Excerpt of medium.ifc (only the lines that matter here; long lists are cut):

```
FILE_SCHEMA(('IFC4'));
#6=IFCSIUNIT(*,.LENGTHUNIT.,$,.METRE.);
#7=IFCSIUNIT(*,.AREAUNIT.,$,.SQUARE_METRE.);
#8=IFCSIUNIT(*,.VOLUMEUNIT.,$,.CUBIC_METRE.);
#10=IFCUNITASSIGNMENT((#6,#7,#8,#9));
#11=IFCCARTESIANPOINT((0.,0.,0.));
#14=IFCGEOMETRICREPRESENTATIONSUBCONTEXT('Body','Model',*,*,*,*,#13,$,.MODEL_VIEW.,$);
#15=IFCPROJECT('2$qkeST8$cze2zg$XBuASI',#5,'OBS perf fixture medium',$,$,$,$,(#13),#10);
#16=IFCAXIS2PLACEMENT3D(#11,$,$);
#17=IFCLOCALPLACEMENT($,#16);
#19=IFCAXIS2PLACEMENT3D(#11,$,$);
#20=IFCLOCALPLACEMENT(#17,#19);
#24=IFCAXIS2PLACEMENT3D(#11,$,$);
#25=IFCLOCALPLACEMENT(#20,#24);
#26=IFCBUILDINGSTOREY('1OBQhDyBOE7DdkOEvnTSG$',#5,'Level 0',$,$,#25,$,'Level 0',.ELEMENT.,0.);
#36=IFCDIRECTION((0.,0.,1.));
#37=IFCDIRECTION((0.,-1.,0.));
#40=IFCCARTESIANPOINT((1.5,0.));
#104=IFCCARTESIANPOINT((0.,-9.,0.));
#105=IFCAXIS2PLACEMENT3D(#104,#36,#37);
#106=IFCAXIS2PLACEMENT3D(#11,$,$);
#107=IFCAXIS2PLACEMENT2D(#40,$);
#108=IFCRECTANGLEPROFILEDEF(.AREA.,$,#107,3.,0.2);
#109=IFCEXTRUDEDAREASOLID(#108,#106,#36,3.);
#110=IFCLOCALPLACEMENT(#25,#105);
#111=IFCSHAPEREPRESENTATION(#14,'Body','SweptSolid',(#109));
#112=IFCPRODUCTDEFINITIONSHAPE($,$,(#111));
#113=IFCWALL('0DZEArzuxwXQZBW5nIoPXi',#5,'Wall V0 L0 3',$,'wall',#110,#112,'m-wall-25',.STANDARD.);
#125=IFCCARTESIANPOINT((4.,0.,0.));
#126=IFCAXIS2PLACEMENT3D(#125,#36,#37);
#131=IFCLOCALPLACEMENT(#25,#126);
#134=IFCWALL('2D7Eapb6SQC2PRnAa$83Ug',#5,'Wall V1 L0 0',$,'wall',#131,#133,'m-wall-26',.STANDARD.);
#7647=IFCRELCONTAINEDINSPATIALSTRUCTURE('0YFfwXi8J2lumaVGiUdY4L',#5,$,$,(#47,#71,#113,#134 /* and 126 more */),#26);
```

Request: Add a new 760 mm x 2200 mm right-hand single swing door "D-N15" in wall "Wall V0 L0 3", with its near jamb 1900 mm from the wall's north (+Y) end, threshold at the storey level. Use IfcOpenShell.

```python
import numpy as np
import ifcopenshell
import ifcopenshell.api.feature
import ifcopenshell.api.geometry
import ifcopenshell.api.root
import ifcopenshell.api.spatial
import ifcopenshell.geom
import ifcopenshell.util.element
import ifcopenshell.util.placement
import ifcopenshell.util.representation
import ifcopenshell.util.shape
import ifcopenshell.util.unit

model = ifcopenshell.open("medium.ifc")
unit_scale = ifcopenshell.util.unit.calculate_unit_scale(model)
settings = ifcopenshell.geom.settings()


def volume(element):
    """Net volume in cubic metres, openings subtracted."""
    shape = ifcopenshell.geom.create_shape(settings, element)
    return ifcopenshell.util.shape.get_volume(shape.geometry)


wall = model.by_guid("0DZEArzuxwXQZBW5nIoPXi")
storey = ifcopenshell.util.element.get_container(wall, ifc_class="IfcBuildingStorey")
context = ifcopenshell.util.representation.get_context(model, "Model", "Body", "MODEL_VIEW")
before = volume(wall)

width, height, from_end, sill = 0.76, 2.2, 1.9, 0.0  # metres

# The wall runs along its own X axis, and the end named is its -X end.
wall_shape = ifcopenshell.geom.create_shape(settings, wall)
x, y, z = ifcopenshell.util.shape.get_vertices(wall_shape.geometry).T
start = x.min() + from_end
face, thickness = float(y.min()), float(y.max() - y.min())
wall_matrix = ifcopenshell.util.placement.get_local_placement(wall.ObjectPlacement)
level = ifcopenshell.util.placement.get_local_placement(storey.ObjectPlacement)[2, 3]


def in_wall(x, y):
    """Placement at x, y metres in the wall's axes, at sill height."""
    matrix = wall_matrix.copy()
    matrix[:, 3] = wall_matrix @ np.array([x / unit_scale, y / unit_scale, 0.0, 1.0])
    matrix[2, 3] = level + sill / unit_scale
    return matrix


# Opening: a box that overshoots both wall faces by 50 mm.
opening = ifcopenshell.api.root.create_entity(model, ifc_class="IfcOpeningElement", predefined_type="OPENING")
box = ifcopenshell.api.geometry.add_wall_representation(
    model, context=context, length=width, height=height, thickness=thickness + 0.1
)
ifcopenshell.api.geometry.assign_representation(model, product=opening, representation=box)
ifcopenshell.api.geometry.edit_object_placement(model, product=opening, matrix=in_wall(start, face - 0.05), is_si=False)
ifcopenshell.api.feature.add_feature(model, feature=opening, element=wall)

door = ifcopenshell.api.root.create_entity(model, ifc_class="IfcDoor", name="D-N15", predefined_type="DOOR")
door.OverallWidth, door.OverallHeight = width / unit_scale, height / unit_scale
door.OperationType = "SINGLE_SWING_RIGHT"
body = ifcopenshell.api.geometry.add_door_representation(
    model,
    context=context,
    overall_width=door.OverallWidth,
    overall_height=door.OverallHeight,
    operation_type="SINGLE_SWING_RIGHT",
    lining_properties={"LiningDepth": thickness / unit_scale, "ThresholdDepth": thickness / unit_scale},
)
ifcopenshell.api.geometry.assign_representation(model, product=door, representation=body)
ifcopenshell.api.spatial.assign_container(model, products=[door], relating_structure=storey)
ifcopenshell.api.feature.add_filling(model, opening=opening, element=door)

# The lining spans the wall, so the door starts at the wall face.
ifcopenshell.api.geometry.edit_object_placement(model, product=door, matrix=in_wall(start, face), is_si=False)

after = volume(wall)

print(f"wall volume {before:.3f} -> {after:.3f} m3")

model.write("medium_updated.ifc")
```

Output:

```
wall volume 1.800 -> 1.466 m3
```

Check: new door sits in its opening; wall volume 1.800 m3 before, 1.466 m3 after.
